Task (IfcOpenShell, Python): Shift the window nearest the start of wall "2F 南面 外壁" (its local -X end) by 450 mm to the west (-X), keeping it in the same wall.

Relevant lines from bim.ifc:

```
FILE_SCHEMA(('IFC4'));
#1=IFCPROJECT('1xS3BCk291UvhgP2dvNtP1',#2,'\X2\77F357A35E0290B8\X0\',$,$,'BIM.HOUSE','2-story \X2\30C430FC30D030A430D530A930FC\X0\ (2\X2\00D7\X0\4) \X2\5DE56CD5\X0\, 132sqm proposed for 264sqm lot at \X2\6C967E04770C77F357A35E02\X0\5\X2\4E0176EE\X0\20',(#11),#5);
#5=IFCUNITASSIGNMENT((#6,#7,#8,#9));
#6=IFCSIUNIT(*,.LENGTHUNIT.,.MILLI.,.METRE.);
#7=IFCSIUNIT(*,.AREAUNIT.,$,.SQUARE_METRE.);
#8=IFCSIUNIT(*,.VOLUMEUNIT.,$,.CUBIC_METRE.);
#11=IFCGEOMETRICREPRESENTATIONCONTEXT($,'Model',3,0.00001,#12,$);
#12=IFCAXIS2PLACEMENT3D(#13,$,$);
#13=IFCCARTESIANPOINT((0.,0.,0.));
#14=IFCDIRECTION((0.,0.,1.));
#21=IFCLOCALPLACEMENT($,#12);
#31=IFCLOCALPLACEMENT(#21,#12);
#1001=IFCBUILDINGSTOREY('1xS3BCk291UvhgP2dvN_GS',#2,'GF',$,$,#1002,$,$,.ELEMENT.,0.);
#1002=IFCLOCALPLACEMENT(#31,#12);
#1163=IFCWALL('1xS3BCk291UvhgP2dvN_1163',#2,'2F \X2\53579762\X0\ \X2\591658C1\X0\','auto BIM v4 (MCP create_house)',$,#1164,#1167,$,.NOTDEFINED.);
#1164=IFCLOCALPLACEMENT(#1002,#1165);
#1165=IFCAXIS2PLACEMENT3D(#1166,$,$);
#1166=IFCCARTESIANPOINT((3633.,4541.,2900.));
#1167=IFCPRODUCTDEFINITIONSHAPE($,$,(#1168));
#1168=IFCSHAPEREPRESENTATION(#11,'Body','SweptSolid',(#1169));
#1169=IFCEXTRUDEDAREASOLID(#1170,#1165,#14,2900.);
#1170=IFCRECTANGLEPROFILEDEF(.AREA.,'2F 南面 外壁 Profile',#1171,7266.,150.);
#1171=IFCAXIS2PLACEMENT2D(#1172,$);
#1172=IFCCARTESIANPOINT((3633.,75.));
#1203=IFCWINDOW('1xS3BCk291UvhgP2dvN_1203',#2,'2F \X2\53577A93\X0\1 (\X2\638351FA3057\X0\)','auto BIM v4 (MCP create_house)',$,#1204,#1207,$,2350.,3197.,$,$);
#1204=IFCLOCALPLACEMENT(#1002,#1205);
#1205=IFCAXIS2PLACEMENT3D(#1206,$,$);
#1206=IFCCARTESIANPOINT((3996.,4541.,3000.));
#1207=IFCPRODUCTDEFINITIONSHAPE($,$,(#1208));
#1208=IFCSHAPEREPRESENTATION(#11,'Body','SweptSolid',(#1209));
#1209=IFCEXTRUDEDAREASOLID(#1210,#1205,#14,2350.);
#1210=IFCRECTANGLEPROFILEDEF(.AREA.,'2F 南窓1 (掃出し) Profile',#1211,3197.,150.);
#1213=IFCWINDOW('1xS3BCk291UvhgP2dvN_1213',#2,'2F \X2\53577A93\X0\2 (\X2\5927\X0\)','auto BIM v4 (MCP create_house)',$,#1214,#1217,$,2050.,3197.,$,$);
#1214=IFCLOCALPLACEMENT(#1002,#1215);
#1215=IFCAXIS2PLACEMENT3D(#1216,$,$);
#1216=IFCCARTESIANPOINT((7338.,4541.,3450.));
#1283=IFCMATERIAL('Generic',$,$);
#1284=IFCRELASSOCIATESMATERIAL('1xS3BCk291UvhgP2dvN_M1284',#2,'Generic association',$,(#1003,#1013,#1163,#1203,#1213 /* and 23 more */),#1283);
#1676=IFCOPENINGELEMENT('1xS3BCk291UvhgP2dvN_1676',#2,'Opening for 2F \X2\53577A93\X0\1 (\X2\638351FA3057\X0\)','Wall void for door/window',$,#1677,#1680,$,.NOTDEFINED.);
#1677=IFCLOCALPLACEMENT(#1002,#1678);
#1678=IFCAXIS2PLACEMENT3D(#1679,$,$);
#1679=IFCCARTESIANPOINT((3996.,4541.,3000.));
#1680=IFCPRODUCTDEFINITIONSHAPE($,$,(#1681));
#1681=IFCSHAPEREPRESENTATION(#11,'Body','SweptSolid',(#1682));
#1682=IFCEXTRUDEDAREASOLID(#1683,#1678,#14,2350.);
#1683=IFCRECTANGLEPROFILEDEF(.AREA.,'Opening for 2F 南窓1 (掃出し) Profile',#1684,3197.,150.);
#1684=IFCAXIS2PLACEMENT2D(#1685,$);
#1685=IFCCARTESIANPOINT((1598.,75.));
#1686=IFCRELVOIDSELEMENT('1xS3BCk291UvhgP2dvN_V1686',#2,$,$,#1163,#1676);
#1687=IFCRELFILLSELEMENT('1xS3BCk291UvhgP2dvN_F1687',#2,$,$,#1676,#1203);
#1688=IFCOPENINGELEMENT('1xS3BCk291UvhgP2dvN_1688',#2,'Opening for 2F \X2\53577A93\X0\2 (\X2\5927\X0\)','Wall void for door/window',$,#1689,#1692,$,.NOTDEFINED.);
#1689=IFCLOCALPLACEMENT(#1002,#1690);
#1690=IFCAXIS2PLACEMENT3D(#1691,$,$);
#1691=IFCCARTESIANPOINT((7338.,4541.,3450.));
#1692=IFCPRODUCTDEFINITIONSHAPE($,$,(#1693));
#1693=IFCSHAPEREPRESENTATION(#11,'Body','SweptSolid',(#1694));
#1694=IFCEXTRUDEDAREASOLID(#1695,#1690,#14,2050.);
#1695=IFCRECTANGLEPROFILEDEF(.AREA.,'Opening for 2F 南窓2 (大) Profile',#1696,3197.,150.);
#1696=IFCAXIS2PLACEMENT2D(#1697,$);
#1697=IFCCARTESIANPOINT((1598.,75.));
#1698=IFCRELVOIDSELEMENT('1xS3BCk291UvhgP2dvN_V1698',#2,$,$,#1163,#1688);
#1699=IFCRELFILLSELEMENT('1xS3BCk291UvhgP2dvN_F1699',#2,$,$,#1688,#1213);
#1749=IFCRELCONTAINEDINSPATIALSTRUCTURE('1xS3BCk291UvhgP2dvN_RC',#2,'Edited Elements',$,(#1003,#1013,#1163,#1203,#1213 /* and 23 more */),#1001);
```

```python
import ifcopenshell
import ifcopenshell.api.geometry
import ifcopenshell.util.placement

model = ifcopenshell.open("bim.ifc")

window = model.by_guid("1xS3BCk291UvhgP2dvN_1203")
opening = window.FillsVoids[0].RelatingOpeningElement
wall = opening.VoidsElements[0].RelatingBuildingElement

wall_matrix = ifcopenshell.util.placement.get_local_placement(wall.ObjectPlacement)
shift = wall_matrix[:3, 0] * -450.0
before = ifcopenshell.util.placement.get_local_placement(window.ObjectPlacement)[:3, 3].copy()

# The window is not placed relative to its opening, so move both.
for product in (opening, window):
    matrix = ifcopenshell.util.placement.get_local_placement(product.ObjectPlacement)
    matrix[:3, 3] += shift
    ifcopenshell.api.geometry.edit_object_placement(model, product=product, matrix=matrix, is_si=False)

after = ifcopenshell.util.placement.get_local_placement(window.ObjectPlacement)[:3, 3]
print("window moved by", (after - before).round(3) + 0.0)

model.write("bim_v2.ifc")
```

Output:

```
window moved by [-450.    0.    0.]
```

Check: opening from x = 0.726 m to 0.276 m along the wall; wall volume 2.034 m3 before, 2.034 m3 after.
